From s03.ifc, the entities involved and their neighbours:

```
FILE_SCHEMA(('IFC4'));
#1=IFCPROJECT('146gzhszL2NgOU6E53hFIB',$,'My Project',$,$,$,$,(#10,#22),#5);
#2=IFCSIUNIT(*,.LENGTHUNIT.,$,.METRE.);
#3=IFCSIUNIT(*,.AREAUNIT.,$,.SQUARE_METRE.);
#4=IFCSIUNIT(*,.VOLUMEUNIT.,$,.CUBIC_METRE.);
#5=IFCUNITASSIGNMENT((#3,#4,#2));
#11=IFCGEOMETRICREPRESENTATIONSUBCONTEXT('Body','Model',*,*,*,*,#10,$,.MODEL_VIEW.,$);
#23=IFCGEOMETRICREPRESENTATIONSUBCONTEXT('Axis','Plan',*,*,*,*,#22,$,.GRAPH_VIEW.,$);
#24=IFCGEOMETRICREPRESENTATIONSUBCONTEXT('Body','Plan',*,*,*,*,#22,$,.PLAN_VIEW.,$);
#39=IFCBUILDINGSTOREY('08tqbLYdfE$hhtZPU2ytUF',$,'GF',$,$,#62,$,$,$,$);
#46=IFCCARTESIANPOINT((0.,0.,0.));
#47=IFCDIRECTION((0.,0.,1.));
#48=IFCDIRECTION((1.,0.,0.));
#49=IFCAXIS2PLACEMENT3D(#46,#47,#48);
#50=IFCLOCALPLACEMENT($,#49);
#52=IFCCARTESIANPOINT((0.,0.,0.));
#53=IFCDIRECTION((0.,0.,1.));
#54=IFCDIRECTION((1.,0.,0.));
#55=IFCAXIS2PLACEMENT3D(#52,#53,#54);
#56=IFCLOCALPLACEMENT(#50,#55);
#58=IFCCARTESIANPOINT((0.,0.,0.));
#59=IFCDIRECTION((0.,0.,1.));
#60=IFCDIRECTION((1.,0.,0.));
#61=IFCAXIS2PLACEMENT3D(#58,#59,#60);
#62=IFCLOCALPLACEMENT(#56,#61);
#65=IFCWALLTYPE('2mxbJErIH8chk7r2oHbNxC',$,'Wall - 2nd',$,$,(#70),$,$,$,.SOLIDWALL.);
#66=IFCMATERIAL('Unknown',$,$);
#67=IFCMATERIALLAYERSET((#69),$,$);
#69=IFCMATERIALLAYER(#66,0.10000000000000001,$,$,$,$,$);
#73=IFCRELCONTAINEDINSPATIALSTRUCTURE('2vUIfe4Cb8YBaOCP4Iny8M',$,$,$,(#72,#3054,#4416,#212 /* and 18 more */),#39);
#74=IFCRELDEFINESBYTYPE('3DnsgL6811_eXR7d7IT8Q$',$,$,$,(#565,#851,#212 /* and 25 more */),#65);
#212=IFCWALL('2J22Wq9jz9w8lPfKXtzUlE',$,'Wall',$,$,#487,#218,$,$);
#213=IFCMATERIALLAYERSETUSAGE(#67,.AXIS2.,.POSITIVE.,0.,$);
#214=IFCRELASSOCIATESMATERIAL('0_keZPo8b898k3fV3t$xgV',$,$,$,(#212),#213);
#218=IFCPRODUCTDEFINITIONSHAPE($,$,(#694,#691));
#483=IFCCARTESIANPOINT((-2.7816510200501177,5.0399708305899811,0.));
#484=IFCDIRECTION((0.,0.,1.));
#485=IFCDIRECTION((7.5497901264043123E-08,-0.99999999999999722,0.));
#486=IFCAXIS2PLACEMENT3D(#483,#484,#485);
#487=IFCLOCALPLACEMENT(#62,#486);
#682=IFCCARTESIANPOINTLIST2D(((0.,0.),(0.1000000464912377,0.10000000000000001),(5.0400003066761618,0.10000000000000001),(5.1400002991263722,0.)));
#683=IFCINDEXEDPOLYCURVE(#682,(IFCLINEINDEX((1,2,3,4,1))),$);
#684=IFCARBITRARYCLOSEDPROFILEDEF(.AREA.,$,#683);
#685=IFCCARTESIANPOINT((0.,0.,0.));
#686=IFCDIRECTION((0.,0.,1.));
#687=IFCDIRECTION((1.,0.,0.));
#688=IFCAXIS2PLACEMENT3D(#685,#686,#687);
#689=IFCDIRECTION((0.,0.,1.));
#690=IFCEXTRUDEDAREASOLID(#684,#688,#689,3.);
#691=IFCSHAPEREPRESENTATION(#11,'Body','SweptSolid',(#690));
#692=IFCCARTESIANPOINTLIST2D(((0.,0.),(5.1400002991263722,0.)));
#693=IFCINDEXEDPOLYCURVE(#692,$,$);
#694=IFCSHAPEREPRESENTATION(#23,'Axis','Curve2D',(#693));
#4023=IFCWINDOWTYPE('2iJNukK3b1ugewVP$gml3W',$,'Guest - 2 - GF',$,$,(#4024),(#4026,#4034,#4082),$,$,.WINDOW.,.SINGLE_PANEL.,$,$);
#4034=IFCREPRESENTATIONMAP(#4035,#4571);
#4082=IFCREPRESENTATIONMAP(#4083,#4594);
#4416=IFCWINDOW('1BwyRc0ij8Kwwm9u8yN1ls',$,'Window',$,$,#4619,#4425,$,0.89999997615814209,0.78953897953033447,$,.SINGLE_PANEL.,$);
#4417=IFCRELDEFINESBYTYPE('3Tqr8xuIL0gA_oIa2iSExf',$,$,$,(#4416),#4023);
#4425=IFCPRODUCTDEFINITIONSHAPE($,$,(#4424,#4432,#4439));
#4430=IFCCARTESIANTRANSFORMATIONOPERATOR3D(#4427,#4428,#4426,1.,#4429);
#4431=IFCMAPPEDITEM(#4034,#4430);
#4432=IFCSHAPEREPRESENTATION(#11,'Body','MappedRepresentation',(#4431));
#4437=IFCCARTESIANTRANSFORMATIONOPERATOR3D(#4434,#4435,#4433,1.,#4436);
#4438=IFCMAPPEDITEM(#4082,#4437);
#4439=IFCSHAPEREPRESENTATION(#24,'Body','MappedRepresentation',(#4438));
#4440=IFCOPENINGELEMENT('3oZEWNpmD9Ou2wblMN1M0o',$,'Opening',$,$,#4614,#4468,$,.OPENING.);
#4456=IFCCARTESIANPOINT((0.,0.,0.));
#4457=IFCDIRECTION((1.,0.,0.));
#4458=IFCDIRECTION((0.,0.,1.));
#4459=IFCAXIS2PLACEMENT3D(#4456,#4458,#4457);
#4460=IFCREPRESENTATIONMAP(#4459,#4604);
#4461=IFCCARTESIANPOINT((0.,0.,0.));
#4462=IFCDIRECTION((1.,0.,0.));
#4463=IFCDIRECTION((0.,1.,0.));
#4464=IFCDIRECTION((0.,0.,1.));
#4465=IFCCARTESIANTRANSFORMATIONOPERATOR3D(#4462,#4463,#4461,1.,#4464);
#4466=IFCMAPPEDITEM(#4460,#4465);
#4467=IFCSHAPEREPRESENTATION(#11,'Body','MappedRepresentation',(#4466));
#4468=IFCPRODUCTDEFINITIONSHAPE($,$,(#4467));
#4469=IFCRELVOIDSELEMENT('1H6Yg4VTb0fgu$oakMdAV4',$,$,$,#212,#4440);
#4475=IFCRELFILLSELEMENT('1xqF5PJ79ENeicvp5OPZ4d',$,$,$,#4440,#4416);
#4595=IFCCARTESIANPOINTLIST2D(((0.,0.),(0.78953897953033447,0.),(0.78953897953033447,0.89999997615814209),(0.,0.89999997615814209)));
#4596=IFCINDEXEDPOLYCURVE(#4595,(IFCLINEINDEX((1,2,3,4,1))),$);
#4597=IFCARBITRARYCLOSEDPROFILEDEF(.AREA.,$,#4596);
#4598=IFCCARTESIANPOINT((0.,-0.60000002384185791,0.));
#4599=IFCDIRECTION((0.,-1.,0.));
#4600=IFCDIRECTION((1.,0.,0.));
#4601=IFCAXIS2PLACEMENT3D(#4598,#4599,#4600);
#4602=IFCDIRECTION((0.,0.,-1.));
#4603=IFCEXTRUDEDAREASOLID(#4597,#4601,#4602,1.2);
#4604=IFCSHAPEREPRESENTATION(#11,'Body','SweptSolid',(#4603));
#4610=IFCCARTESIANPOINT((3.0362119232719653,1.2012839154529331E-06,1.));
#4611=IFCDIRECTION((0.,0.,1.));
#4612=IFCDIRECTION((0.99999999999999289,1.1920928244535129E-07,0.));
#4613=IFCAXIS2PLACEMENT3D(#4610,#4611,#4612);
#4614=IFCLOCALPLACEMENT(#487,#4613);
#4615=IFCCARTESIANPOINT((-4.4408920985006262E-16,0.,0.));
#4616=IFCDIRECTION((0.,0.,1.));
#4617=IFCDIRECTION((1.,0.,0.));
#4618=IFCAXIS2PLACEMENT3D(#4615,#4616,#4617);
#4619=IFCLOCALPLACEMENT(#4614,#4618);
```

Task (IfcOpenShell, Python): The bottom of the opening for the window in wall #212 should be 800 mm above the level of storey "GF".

```python
import numpy as np
import ifcopenshell
import ifcopenshell.api.geometry
import ifcopenshell.geom
import ifcopenshell.util.element
import ifcopenshell.util.placement
import ifcopenshell.util.shape
import ifcopenshell.util.unit

model = ifcopenshell.open("s03.ifc")
unit_scale = ifcopenshell.util.unit.calculate_unit_scale(model)

window = model.by_guid("1BwyRc0ij8Kwwm9u8yN1ls")
opening = window.FillsVoids[0].RelatingOpeningElement
storey = ifcopenshell.util.element.get_container(window, ifc_class="IfcBuildingStorey")
level = ifcopenshell.util.placement.get_local_placement(storey.ObjectPlacement)[2, 3]

# The opening's origin need not be at the sill, so measure its lowest point.
shape = ifcopenshell.geom.create_shape(ifcopenshell.geom.settings(), opening)
bottom = ifcopenshell.util.shape.get_shape_bottom_elevation(shape, shape.geometry) / unit_scale
dz = level + 0.8 / unit_scale - bottom

shift = np.array([0.0, 0.0, dz])
# The window is placed relative to its opening, so it follows when the opening moves.
matrix = ifcopenshell.util.placement.get_local_placement(opening.ObjectPlacement)
matrix[:3, 3] += shift
ifcopenshell.api.geometry.edit_object_placement(
    model, product=opening, matrix=matrix, is_si=False, should_transform_children=True
)

print(f"moved by {dz * unit_scale:+.3f} m")

model.write("s03_v2.ifc")
```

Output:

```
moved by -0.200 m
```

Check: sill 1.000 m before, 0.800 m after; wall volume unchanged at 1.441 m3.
